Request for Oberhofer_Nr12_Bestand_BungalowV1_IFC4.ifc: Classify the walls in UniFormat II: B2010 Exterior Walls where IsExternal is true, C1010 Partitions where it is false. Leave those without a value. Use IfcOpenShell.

First a look at what the model holds.

```python
import ifcopenshell
import ifcopenshell.util.element

model = ifcopenshell.open("Oberhofer_Nr12_Bestand_BungalowV1_IFC4.ifc")
print(model.schema)
print("classifications:", [c.Name for c in model.by_type("IfcClassification")])
values = [ifcopenshell.util.element.get_pset(e, "Pset_WallCommon", "IsExternal") for e in model.by_type("IfcWall")]
for value in (True, False, None):
    print("IsExternal", value, values.count(value))
```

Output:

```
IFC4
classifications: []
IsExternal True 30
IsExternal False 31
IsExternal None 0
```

```python
import ifcopenshell
import ifcopenshell.api.classification
import ifcopenshell.util.element

model = ifcopenshell.open("Oberhofer_Nr12_Bestand_BungalowV1_IFC4.ifc")

system = ifcopenshell.api.classification.add_classification(model, classification="UniFormat II")

walls = model.by_type("IfcWall")
external = {e: ifcopenshell.util.element.get_pset(e, "Pset_WallCommon", "IsExternal") for e in walls}
for flag, code, name in ((True, "B2010", "Exterior Walls"), (False, "C1010", "Partitions")):
    products = [e for e in walls if external[e] is flag]
    ifcopenshell.api.classification.add_reference(
        model, products=products, classification=system, identification=code, name=name
    )
    print(code, len(products))

model.write("Oberhofer_Nr12_Bestand_BungalowV1_IFC4_rev.ifc")
```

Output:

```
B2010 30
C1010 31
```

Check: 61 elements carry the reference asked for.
